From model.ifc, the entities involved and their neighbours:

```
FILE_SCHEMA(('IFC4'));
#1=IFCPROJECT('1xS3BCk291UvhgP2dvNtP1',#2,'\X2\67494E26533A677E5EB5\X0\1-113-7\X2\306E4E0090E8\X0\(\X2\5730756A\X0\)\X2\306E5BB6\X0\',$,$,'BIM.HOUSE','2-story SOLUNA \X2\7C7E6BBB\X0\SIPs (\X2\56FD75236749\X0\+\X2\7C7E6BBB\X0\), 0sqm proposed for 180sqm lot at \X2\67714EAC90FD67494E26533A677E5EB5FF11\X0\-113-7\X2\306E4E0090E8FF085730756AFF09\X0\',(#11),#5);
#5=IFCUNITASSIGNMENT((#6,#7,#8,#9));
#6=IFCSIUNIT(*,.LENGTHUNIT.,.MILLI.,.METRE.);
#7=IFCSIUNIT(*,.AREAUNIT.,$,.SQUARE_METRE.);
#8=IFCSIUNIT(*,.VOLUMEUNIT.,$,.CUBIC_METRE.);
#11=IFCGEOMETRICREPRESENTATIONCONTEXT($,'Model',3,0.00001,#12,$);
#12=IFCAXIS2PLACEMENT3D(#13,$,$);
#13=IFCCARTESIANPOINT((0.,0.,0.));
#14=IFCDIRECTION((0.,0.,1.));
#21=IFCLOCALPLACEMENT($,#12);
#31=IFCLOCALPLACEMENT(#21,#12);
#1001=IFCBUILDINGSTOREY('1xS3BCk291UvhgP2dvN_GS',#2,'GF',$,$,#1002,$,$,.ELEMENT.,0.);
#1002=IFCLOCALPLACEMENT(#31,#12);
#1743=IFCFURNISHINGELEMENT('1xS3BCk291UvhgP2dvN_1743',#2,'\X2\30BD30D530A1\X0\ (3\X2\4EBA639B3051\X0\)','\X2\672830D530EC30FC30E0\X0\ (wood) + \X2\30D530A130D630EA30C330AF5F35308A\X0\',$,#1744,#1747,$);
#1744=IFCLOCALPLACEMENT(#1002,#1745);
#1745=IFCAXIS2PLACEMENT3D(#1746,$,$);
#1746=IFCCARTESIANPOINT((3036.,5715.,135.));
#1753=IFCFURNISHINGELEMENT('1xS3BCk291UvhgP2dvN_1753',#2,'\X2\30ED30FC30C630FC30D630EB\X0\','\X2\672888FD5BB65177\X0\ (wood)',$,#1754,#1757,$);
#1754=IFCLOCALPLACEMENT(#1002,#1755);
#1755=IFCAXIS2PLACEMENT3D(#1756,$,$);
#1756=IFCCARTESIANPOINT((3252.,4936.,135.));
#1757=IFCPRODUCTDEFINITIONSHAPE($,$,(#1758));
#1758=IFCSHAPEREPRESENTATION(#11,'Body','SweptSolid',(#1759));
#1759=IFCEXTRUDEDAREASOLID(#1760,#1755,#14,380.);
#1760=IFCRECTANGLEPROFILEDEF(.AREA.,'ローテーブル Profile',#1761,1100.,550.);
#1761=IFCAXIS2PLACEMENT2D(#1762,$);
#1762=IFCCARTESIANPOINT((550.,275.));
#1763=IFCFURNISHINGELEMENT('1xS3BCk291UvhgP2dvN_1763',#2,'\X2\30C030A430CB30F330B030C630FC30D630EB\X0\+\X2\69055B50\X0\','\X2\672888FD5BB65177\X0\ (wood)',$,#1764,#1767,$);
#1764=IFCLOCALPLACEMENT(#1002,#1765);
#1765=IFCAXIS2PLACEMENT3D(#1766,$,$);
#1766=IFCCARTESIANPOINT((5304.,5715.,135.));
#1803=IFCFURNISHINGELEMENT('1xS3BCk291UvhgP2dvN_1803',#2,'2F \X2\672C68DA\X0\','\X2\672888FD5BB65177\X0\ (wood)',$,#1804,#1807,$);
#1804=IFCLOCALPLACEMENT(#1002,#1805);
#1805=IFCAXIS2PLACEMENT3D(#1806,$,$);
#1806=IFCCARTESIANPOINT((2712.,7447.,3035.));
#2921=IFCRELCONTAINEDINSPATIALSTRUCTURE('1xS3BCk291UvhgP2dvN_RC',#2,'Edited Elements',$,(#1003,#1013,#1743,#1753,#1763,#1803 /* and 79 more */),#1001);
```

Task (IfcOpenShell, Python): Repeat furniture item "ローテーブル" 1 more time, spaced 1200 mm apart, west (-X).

```python
import numpy as np
import ifcopenshell
import ifcopenshell.api.geometry
import ifcopenshell.api.root
import ifcopenshell.util.element
import ifcopenshell.util.placement
import ifcopenshell.util.unit

model = ifcopenshell.open("model.ifc")
unit_scale = ifcopenshell.util.unit.calculate_unit_scale(model)


def reuse_history(source, copy):
    """copy_class also copies each property set's owner history, people and application; keep the originals."""
    for rel in copy.IsDefinedBy:
        if rel.is_a("IfcRelDefinesByProperties") and (history := rel.RelatingPropertyDefinition.OwnerHistory):
            rel.RelatingPropertyDefinition.OwnerHistory = source.OwnerHistory
            ifcopenshell.util.element.remove_deep2(model, history)


source = model.by_id(1753)
base = ifcopenshell.util.placement.get_local_placement(source.ObjectPlacement)
step = np.array([-1.0, 0.0, 0.0]) * 1.2 / unit_scale

for i in range(1, 2):
    copy = ifcopenshell.api.root.copy_class(model, product=source)
    copy.Representation = ifcopenshell.util.element.copy_deep(
        model, source.Representation, exclude=["IfcGeometricRepresentationContext", "IfcRepresentationMap"]
    )
    reuse_history(source, copy)
    matrix = base.copy()
    matrix[:3, 3] += i * step
    print("added at", matrix[:3, 3].round(3) + 0.0)
    ifcopenshell.api.geometry.edit_object_placement(model, product=copy, matrix=matrix, is_si=False)

model.write("model-out.ifc")
```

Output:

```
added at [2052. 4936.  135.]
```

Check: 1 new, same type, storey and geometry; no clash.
